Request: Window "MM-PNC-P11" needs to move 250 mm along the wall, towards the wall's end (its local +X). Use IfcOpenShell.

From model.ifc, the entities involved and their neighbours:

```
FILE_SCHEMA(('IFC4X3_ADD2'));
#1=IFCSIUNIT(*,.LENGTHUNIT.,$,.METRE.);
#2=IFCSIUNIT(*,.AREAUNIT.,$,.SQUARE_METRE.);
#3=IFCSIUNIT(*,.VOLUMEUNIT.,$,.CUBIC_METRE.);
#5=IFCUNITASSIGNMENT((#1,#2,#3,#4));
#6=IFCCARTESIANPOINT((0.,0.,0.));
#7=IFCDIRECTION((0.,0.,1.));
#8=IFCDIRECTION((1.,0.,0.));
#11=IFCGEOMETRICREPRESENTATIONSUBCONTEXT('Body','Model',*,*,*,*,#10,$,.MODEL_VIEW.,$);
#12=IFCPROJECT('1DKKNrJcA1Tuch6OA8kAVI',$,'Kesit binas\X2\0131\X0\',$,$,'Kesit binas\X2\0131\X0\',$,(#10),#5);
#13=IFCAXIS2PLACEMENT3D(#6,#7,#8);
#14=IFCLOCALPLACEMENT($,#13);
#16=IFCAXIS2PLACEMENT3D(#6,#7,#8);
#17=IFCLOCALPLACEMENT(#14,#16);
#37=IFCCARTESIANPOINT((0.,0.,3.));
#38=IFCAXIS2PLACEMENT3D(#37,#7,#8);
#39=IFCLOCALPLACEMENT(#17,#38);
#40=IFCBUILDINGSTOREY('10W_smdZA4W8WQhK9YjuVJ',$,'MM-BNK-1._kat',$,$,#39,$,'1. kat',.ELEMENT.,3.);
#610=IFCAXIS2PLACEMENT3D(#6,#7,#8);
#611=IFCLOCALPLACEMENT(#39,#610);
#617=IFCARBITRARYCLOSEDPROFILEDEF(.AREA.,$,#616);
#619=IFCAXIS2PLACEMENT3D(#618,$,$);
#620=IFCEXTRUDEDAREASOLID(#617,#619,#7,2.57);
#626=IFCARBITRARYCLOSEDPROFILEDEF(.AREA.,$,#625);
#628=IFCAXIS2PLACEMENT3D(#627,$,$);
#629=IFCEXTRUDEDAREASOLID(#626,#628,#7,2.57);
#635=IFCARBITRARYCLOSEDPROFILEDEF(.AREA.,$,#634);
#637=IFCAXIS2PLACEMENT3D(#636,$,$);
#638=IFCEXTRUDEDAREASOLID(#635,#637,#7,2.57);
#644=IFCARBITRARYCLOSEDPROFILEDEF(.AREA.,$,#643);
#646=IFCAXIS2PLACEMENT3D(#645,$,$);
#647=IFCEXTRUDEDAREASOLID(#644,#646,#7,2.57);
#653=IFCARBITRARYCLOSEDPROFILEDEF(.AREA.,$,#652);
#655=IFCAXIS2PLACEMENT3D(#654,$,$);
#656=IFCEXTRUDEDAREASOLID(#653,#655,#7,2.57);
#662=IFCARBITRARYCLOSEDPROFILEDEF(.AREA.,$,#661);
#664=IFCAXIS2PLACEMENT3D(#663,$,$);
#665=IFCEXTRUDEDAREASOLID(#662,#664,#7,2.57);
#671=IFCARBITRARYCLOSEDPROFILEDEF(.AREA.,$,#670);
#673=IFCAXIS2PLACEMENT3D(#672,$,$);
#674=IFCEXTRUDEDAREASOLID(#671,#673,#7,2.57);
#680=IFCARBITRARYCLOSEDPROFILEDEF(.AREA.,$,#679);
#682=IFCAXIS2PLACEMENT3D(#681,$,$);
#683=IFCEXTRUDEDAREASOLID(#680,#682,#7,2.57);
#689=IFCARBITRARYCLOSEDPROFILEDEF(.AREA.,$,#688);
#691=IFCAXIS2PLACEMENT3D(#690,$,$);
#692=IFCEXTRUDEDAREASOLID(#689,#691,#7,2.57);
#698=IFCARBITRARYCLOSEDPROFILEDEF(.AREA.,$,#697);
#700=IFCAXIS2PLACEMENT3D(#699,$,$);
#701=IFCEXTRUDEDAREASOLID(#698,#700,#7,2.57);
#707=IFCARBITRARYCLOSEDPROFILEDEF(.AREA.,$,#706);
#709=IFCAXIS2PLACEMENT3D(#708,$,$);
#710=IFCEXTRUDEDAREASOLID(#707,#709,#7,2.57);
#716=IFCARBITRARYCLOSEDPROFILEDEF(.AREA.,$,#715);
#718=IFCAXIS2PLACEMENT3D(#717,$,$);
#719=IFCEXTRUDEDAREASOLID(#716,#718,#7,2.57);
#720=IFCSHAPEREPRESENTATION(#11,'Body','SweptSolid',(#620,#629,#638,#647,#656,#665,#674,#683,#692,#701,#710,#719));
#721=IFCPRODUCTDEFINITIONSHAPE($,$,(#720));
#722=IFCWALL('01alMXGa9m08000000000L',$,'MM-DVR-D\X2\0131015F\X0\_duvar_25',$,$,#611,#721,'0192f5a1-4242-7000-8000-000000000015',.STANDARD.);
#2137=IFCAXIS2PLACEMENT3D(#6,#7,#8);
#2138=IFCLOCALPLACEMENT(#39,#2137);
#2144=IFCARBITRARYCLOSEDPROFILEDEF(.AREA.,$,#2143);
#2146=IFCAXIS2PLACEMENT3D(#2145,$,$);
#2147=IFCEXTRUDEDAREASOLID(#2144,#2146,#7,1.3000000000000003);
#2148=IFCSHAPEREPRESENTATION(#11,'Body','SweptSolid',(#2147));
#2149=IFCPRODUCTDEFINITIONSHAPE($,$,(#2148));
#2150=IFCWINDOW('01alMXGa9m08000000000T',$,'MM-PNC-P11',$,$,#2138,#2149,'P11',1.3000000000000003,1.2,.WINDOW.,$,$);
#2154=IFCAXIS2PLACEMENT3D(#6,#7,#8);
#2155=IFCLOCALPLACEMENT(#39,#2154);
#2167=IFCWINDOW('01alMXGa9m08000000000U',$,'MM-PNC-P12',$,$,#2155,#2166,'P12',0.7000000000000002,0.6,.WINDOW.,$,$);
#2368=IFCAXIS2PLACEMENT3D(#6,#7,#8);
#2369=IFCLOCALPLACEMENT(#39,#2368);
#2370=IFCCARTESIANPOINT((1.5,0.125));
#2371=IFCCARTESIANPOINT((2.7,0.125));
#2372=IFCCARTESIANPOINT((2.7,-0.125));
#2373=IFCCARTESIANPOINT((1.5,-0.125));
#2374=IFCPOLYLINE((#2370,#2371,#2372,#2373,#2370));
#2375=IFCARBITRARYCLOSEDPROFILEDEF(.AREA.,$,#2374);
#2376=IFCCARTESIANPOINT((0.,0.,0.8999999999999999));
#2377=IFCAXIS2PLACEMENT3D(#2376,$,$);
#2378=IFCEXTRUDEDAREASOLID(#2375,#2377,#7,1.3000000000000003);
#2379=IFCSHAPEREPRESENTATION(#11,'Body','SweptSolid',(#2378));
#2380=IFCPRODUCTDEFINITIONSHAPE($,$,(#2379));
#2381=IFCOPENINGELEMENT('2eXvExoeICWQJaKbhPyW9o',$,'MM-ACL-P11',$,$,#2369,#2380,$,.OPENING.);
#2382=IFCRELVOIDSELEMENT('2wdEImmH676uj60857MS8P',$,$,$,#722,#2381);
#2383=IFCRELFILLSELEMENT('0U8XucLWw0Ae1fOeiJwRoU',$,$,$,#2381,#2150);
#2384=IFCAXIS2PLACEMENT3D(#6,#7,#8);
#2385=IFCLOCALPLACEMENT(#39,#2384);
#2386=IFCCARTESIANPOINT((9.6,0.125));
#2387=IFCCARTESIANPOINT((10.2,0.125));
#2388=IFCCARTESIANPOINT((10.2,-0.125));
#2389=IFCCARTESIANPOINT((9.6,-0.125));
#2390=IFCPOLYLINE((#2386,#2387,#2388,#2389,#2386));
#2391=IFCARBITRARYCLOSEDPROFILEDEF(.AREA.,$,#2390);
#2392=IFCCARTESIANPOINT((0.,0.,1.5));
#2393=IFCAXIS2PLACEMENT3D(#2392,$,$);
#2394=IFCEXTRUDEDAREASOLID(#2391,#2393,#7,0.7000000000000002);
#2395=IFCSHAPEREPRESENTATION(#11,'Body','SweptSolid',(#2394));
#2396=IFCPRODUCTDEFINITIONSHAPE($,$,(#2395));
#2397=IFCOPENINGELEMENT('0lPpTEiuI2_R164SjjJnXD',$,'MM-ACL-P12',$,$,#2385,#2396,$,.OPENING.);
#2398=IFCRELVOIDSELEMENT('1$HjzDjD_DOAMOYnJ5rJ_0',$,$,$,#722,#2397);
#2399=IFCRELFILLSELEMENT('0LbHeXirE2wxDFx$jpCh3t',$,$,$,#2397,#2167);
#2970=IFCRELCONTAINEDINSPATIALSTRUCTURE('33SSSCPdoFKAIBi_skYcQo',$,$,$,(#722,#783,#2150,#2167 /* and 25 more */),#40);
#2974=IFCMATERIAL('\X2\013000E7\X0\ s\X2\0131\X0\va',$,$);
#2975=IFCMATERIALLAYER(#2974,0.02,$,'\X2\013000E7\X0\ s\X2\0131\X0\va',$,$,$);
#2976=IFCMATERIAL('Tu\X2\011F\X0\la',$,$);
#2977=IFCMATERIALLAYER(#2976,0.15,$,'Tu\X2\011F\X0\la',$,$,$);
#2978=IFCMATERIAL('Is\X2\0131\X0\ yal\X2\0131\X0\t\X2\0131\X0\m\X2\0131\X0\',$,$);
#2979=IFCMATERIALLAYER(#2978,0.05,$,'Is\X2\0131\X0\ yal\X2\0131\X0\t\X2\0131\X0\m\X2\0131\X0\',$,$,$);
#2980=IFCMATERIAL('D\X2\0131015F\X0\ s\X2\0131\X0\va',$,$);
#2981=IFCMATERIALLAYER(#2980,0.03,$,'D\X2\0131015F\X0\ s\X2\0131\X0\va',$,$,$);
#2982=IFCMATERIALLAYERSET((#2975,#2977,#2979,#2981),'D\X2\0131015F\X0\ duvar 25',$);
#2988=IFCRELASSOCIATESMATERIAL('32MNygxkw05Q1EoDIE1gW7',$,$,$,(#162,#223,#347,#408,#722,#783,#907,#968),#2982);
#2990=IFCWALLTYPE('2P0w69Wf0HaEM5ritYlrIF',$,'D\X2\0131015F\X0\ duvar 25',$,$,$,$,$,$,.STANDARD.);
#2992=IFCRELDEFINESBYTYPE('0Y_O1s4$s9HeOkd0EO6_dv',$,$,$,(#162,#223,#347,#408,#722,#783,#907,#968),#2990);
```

```python
import ifcopenshell
import ifcopenshell.api.geometry
import ifcopenshell.util.placement

model = ifcopenshell.open("model.ifc")

window = model.by_id(2150)
opening = window.FillsVoids[0].RelatingOpeningElement
wall = opening.VoidsElements[0].RelatingBuildingElement

wall_matrix = ifcopenshell.util.placement.get_local_placement(wall.ObjectPlacement)
shift = wall_matrix[:3, 0] * 0.25
before = ifcopenshell.util.placement.get_local_placement(window.ObjectPlacement)[:3, 3].copy()

# The window is not placed relative to its opening, so move both.
for product in (opening, window):
    matrix = ifcopenshell.util.placement.get_local_placement(product.ObjectPlacement)
    matrix[:3, 3] += shift
    ifcopenshell.api.geometry.edit_object_placement(model, product=product, matrix=matrix, is_si=False)

after = ifcopenshell.util.placement.get_local_placement(window.ObjectPlacement)[:3, 3]
print("window moved by", (after - before).round(3) + 0.0)

model.write("model_v2.ifc")
```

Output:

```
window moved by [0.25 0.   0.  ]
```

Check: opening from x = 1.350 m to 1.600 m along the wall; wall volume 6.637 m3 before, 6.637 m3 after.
